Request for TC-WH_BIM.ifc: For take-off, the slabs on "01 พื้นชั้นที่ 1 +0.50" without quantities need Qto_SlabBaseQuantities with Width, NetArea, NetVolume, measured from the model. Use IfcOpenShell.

First a look at what the model holds.

```python
import ifcopenshell
import ifcopenshell.util.element
import ifcopenshell.util.unit

model = ifcopenshell.open("TC-WH_BIM.ifc")
print(model.schema)
for unit_type in ("LENGTHUNIT", "AREAUNIT", "VOLUMEUNIT"):
    print(unit_type, ifcopenshell.util.unit.calculate_unit_scale(model, unit_type))
storey = next(s for s in model.by_type("IfcBuildingStorey") if s.Name == "01 พื้นชั้นที่ 1 +0.50")
slabs = [e for e in ifcopenshell.util.element.get_decomposition(storey) if e.is_a("IfcSlab")]
for e in sorted(slabs, key=lambda e: e.id()):
    print(e.id(), e.is_a(), e.Name, list(ifcopenshell.util.element.get_psets(e, qtos_only=True)), sep=" | ")
```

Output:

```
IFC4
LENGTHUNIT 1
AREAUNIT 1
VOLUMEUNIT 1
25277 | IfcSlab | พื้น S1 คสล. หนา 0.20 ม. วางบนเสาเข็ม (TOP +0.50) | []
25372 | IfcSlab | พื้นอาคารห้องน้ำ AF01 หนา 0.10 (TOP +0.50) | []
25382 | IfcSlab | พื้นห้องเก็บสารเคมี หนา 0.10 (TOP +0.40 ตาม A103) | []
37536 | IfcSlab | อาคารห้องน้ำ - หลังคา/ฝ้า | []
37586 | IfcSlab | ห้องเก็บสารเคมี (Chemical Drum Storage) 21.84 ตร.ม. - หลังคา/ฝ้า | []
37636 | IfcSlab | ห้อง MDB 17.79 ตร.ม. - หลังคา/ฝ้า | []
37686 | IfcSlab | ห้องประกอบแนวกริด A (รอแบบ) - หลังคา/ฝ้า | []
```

```python
import ifcopenshell
import ifcopenshell.api.pset
import ifcopenshell.geom
import ifcopenshell.util.element
import ifcopenshell.util.shape
import ifcopenshell.util.unit

model = ifcopenshell.open("TC-WH_BIM.ifc")
unit_scale = ifcopenshell.util.unit.calculate_unit_scale(model)
area_scale = ifcopenshell.util.unit.calculate_unit_scale(model, "AREAUNIT")
volume_scale = ifcopenshell.util.unit.calculate_unit_scale(model, "VOLUMEUNIT")
settings = ifcopenshell.geom.settings()

storey = next(s for s in model.by_type("IfcBuildingStorey") if s.Name == "01 พื้นชั้นที่ 1 +0.50")
slabs = [e for e in ifcopenshell.util.element.get_decomposition(storey) if e.is_a("IfcSlab")]

for e in sorted(slabs, key=lambda e: e.id()):
    if ifcopenshell.util.element.get_psets(e, qtos_only=True, should_inherit=False):
        continue
    # Geometry comes back in metres, in the element's own axes.
    shape = ifcopenshell.geom.create_shape(settings, e)
    values = {
        "Width": ifcopenshell.util.shape.get_z(shape.geometry) / unit_scale,
        "NetArea": ifcopenshell.util.shape.get_footprint_area(shape.geometry) / area_scale,
        "NetVolume": ifcopenshell.util.shape.get_volume(shape.geometry) / volume_scale,
    }
    qto = ifcopenshell.api.pset.add_qto(model, product=e, name="Qto_SlabBaseQuantities")
    ifcopenshell.api.pset.edit_qto(model, qto=qto, properties=values)
    print(e.id(), {k: round(v, 3) for k, v in values.items()})

model.write("TC-WH_BIM-out.ifc")
```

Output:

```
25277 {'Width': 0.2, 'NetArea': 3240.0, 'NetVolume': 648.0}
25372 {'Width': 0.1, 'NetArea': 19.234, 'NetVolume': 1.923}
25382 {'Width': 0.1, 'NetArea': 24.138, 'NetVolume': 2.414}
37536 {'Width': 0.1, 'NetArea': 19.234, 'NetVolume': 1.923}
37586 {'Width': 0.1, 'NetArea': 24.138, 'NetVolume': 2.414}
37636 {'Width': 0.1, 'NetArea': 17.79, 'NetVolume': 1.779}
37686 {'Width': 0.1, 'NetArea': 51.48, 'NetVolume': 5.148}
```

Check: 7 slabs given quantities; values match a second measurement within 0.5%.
